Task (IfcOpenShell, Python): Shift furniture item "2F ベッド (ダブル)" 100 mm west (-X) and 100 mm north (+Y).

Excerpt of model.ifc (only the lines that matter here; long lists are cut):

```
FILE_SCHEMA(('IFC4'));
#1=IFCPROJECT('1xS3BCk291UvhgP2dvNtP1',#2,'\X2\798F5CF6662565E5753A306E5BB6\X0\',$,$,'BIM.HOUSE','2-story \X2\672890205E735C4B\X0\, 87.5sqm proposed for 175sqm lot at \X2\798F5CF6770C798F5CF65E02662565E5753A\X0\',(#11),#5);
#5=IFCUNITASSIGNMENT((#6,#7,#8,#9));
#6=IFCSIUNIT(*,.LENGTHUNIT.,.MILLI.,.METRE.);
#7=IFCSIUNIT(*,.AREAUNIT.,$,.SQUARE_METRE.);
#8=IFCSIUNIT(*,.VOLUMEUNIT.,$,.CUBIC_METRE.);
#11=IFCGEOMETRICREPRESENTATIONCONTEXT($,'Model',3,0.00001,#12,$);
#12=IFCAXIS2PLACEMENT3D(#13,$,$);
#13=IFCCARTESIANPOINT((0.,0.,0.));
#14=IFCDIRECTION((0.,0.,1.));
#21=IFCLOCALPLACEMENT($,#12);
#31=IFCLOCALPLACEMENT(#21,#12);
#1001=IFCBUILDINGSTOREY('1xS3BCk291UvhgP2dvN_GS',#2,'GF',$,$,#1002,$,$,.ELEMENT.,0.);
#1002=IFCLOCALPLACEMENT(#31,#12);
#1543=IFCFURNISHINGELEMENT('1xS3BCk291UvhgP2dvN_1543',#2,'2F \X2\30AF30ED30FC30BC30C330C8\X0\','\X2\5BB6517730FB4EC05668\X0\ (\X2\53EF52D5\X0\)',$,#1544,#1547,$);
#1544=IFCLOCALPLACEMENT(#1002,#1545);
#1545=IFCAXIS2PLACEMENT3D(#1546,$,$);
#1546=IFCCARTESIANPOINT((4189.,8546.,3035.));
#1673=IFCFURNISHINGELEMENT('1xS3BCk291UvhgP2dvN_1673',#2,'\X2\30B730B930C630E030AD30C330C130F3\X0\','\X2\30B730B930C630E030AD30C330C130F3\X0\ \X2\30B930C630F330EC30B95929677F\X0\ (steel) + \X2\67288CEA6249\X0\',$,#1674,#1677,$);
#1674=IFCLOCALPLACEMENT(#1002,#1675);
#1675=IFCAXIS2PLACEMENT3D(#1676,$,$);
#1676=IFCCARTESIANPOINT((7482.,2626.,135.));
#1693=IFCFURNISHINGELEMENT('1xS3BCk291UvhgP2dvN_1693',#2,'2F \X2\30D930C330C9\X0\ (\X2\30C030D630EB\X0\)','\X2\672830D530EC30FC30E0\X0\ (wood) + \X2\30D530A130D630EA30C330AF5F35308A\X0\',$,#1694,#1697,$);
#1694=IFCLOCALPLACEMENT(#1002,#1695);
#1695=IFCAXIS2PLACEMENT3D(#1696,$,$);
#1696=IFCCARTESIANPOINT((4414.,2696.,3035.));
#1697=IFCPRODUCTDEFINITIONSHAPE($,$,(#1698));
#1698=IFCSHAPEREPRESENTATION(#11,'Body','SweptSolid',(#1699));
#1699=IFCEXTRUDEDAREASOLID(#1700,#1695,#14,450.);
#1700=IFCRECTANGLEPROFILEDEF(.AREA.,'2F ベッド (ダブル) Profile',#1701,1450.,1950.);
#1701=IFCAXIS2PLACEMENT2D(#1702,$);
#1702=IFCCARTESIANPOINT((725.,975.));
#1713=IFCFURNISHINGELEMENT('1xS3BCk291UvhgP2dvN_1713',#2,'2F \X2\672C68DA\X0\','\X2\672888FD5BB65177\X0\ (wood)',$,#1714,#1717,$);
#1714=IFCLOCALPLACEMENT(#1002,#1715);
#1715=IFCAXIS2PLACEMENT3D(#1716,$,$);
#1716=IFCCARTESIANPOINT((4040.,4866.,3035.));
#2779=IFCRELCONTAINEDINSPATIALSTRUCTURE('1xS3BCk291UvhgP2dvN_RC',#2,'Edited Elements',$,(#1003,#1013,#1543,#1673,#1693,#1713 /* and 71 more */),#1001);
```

```python
import ifcopenshell
import ifcopenshell.api.geometry
import ifcopenshell.util.placement
import ifcopenshell.util.unit

model = ifcopenshell.open("model.ifc")
unit_scale = ifcopenshell.util.unit.calculate_unit_scale(model)

item = model.by_guid("1xS3BCk291UvhgP2dvN_1693")
matrix = ifcopenshell.util.placement.get_local_placement(item.ObjectPlacement)
matrix[0, 3] -= 0.1 / unit_scale
matrix[1, 3] += 0.1 / unit_scale
ifcopenshell.api.geometry.edit_object_placement(model, product=item, matrix=matrix, is_si=False)

print(ifcopenshell.util.placement.get_local_placement(item.ObjectPlacement).round(3) + 0.0)

model.write("model_updated.ifc")
```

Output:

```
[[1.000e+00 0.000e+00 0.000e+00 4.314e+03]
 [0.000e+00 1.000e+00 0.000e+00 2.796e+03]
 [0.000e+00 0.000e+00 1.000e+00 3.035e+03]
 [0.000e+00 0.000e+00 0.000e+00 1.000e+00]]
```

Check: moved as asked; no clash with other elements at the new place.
